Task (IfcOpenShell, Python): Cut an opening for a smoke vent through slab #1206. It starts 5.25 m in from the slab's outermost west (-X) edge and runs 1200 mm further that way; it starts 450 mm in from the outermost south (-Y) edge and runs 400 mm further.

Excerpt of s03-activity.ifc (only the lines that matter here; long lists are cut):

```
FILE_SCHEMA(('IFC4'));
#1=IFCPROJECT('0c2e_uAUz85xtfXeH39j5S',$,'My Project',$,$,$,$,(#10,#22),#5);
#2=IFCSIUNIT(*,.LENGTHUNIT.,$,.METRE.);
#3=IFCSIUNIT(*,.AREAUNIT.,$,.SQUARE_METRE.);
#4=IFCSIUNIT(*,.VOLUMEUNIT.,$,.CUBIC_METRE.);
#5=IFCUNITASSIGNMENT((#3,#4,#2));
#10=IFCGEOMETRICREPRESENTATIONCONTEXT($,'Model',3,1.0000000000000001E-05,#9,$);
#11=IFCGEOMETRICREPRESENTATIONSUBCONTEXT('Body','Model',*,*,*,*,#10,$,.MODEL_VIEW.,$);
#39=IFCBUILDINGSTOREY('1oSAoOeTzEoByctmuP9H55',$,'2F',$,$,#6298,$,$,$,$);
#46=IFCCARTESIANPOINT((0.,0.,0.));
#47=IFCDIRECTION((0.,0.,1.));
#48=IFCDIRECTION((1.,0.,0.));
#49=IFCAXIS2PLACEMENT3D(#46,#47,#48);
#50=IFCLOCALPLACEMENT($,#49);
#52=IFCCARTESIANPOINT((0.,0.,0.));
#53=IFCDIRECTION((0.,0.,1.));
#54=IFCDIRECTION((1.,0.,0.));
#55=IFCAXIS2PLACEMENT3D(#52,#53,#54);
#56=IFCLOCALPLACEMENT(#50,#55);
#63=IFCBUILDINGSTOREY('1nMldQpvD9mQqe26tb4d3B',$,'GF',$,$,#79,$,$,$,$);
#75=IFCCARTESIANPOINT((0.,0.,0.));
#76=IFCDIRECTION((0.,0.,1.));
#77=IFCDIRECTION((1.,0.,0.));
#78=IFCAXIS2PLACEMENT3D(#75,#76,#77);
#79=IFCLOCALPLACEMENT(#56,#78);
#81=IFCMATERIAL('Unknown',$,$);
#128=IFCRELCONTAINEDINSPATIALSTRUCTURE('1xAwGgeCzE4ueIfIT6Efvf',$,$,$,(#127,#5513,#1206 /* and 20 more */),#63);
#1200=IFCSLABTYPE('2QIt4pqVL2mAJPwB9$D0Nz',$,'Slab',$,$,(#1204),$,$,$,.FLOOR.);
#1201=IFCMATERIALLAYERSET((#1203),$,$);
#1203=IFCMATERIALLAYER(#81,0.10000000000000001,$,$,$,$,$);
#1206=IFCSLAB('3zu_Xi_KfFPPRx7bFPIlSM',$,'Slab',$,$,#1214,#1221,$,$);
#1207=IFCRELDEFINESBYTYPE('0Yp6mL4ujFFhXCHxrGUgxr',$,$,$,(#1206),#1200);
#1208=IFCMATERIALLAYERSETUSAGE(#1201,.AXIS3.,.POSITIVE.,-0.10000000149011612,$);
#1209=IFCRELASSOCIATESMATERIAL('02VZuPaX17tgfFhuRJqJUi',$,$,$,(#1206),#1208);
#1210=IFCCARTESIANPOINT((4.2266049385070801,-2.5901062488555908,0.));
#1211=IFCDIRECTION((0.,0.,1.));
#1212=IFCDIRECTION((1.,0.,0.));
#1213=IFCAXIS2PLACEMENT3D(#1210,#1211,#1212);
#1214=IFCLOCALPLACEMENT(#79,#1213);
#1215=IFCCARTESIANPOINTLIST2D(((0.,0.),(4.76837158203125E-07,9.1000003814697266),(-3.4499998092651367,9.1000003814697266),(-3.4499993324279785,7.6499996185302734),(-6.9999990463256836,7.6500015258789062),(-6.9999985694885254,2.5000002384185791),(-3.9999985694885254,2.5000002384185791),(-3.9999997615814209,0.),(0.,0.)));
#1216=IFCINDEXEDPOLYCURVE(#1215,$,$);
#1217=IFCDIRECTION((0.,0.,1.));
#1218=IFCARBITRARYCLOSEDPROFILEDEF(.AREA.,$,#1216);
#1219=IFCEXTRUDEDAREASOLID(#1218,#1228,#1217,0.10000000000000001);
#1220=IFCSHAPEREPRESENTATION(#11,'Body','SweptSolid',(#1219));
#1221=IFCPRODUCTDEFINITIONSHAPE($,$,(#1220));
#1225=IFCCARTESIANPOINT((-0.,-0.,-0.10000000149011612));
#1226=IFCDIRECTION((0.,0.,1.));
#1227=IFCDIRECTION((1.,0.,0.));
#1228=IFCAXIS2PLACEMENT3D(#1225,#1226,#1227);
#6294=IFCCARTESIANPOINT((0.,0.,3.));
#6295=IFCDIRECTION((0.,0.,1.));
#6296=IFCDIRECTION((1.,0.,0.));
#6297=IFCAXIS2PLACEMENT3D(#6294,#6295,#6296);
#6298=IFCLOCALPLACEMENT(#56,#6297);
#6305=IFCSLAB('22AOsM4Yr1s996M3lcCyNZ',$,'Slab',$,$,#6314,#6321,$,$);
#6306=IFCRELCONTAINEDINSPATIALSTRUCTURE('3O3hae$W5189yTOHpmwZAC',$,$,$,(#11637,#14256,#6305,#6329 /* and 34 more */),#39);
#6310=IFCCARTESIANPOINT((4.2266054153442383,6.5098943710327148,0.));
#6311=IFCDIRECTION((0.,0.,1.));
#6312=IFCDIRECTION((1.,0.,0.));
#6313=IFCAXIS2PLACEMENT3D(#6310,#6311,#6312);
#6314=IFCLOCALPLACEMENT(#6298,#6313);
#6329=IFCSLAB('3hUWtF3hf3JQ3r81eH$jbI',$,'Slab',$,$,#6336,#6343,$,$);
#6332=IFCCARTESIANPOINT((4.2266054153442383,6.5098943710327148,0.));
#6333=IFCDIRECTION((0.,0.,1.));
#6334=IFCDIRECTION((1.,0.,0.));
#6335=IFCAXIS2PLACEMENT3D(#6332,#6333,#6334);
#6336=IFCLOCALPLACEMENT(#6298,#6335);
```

```python
import numpy as np
import ifcopenshell
import ifcopenshell.api.feature
import ifcopenshell.api.geometry
import ifcopenshell.api.root
import ifcopenshell.geom
import ifcopenshell.util.placement
import ifcopenshell.util.representation
import ifcopenshell.util.shape
import ifcopenshell.util.unit

model = ifcopenshell.open("s03-activity.ifc")
unit_scale = ifcopenshell.util.unit.calculate_unit_scale(model)
settings = ifcopenshell.geom.settings()


def volume(element):
    """Net volume in cubic metres, openings subtracted."""
    shape = ifcopenshell.geom.create_shape(settings, element)
    return ifcopenshell.util.shape.get_volume(shape.geometry)


slab = model.by_guid("3zu_Xi_KfFPPRx7bFPIlSM")
before = volume(slab)

# Extent in the slab's own axes, in metres. The edges named are its -X and -Y sides.
slab_shape = ifcopenshell.geom.create_shape(settings, slab)
vertices = ifcopenshell.util.shape.get_vertices(slab_shape.geometry)
x_min, y_min, bottom = vertices.min(axis=0)
top = vertices[:, 2].max()

opening = ifcopenshell.api.root.create_entity(model, ifc_class="IfcOpeningElement", name="Smoke vent opening", predefined_type="OPENING")
context = ifcopenshell.util.representation.get_context(model, "Model", "Body", "MODEL_VIEW")
width, depth = 1.2, 0.4
outline = [(0.0, 0.0), (width, 0.0), (width, depth), (0.0, depth), (0.0, 0.0)]
# Overshoot both faces by 50 mm so the cut is clean.
shape = ifcopenshell.api.geometry.add_slab_representation(
    model, context=context, depth=top - bottom + 0.1, polyline=outline
)
ifcopenshell.api.geometry.assign_representation(model, product=opening, representation=shape)

matrix = ifcopenshell.util.placement.get_local_placement(slab.ObjectPlacement)
matrix[:, 3] = matrix @ np.append(np.array([x_min + 5.25, y_min + 0.45, bottom - 0.05]) / unit_scale, 1.0)
ifcopenshell.api.geometry.edit_object_placement(model, product=opening, matrix=matrix, is_si=False)
ifcopenshell.api.feature.add_feature(model, feature=opening, element=slab)

after = volume(slab)

print(f"slab volume {before:.3f} -> {after:.3f} m3")

model.write("s03-activity-out.ifc")
```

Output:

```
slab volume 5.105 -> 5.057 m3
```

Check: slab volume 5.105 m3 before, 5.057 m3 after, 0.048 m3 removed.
